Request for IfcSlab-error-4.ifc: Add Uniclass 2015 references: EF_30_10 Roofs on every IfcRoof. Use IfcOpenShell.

First a look at what the model holds.

```python
import ifcopenshell

model = ifcopenshell.open("IfcSlab-error-4.ifc")
print(model.schema)
print("classifications:", [c.Name for c in model.by_type("IfcClassification")])
for ifc_class in ("IfcDoor", "IfcRoof", "IfcStair", "IfcWall", "IfcWindow"):
    print(ifc_class, len(model.by_type(ifc_class)))
```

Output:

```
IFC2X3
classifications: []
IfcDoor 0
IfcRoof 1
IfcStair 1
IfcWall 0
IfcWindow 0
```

```python
import ifcopenshell
import ifcopenshell.api.classification

model = ifcopenshell.open("IfcSlab-error-4.ifc")

# IFC2X3 requires Source and Edition and has no link from the project to the system.
system = model.create_entity("IfcClassification", Source="NBS", Edition="2015", Name="Uniclass 2015")

codes = {
    "IfcRoof": ("EF_30_10", "Roofs"),
}
for ifc_class, (code, name) in codes.items():
    products = model.by_type(ifc_class)
    ifcopenshell.api.classification.add_reference(
        model, products=products, classification=system, identification=code, name=name
    )
    print(code, len(products))

model.write("IfcSlab-error-4_rev.ifc")
```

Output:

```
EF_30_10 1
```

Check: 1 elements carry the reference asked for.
